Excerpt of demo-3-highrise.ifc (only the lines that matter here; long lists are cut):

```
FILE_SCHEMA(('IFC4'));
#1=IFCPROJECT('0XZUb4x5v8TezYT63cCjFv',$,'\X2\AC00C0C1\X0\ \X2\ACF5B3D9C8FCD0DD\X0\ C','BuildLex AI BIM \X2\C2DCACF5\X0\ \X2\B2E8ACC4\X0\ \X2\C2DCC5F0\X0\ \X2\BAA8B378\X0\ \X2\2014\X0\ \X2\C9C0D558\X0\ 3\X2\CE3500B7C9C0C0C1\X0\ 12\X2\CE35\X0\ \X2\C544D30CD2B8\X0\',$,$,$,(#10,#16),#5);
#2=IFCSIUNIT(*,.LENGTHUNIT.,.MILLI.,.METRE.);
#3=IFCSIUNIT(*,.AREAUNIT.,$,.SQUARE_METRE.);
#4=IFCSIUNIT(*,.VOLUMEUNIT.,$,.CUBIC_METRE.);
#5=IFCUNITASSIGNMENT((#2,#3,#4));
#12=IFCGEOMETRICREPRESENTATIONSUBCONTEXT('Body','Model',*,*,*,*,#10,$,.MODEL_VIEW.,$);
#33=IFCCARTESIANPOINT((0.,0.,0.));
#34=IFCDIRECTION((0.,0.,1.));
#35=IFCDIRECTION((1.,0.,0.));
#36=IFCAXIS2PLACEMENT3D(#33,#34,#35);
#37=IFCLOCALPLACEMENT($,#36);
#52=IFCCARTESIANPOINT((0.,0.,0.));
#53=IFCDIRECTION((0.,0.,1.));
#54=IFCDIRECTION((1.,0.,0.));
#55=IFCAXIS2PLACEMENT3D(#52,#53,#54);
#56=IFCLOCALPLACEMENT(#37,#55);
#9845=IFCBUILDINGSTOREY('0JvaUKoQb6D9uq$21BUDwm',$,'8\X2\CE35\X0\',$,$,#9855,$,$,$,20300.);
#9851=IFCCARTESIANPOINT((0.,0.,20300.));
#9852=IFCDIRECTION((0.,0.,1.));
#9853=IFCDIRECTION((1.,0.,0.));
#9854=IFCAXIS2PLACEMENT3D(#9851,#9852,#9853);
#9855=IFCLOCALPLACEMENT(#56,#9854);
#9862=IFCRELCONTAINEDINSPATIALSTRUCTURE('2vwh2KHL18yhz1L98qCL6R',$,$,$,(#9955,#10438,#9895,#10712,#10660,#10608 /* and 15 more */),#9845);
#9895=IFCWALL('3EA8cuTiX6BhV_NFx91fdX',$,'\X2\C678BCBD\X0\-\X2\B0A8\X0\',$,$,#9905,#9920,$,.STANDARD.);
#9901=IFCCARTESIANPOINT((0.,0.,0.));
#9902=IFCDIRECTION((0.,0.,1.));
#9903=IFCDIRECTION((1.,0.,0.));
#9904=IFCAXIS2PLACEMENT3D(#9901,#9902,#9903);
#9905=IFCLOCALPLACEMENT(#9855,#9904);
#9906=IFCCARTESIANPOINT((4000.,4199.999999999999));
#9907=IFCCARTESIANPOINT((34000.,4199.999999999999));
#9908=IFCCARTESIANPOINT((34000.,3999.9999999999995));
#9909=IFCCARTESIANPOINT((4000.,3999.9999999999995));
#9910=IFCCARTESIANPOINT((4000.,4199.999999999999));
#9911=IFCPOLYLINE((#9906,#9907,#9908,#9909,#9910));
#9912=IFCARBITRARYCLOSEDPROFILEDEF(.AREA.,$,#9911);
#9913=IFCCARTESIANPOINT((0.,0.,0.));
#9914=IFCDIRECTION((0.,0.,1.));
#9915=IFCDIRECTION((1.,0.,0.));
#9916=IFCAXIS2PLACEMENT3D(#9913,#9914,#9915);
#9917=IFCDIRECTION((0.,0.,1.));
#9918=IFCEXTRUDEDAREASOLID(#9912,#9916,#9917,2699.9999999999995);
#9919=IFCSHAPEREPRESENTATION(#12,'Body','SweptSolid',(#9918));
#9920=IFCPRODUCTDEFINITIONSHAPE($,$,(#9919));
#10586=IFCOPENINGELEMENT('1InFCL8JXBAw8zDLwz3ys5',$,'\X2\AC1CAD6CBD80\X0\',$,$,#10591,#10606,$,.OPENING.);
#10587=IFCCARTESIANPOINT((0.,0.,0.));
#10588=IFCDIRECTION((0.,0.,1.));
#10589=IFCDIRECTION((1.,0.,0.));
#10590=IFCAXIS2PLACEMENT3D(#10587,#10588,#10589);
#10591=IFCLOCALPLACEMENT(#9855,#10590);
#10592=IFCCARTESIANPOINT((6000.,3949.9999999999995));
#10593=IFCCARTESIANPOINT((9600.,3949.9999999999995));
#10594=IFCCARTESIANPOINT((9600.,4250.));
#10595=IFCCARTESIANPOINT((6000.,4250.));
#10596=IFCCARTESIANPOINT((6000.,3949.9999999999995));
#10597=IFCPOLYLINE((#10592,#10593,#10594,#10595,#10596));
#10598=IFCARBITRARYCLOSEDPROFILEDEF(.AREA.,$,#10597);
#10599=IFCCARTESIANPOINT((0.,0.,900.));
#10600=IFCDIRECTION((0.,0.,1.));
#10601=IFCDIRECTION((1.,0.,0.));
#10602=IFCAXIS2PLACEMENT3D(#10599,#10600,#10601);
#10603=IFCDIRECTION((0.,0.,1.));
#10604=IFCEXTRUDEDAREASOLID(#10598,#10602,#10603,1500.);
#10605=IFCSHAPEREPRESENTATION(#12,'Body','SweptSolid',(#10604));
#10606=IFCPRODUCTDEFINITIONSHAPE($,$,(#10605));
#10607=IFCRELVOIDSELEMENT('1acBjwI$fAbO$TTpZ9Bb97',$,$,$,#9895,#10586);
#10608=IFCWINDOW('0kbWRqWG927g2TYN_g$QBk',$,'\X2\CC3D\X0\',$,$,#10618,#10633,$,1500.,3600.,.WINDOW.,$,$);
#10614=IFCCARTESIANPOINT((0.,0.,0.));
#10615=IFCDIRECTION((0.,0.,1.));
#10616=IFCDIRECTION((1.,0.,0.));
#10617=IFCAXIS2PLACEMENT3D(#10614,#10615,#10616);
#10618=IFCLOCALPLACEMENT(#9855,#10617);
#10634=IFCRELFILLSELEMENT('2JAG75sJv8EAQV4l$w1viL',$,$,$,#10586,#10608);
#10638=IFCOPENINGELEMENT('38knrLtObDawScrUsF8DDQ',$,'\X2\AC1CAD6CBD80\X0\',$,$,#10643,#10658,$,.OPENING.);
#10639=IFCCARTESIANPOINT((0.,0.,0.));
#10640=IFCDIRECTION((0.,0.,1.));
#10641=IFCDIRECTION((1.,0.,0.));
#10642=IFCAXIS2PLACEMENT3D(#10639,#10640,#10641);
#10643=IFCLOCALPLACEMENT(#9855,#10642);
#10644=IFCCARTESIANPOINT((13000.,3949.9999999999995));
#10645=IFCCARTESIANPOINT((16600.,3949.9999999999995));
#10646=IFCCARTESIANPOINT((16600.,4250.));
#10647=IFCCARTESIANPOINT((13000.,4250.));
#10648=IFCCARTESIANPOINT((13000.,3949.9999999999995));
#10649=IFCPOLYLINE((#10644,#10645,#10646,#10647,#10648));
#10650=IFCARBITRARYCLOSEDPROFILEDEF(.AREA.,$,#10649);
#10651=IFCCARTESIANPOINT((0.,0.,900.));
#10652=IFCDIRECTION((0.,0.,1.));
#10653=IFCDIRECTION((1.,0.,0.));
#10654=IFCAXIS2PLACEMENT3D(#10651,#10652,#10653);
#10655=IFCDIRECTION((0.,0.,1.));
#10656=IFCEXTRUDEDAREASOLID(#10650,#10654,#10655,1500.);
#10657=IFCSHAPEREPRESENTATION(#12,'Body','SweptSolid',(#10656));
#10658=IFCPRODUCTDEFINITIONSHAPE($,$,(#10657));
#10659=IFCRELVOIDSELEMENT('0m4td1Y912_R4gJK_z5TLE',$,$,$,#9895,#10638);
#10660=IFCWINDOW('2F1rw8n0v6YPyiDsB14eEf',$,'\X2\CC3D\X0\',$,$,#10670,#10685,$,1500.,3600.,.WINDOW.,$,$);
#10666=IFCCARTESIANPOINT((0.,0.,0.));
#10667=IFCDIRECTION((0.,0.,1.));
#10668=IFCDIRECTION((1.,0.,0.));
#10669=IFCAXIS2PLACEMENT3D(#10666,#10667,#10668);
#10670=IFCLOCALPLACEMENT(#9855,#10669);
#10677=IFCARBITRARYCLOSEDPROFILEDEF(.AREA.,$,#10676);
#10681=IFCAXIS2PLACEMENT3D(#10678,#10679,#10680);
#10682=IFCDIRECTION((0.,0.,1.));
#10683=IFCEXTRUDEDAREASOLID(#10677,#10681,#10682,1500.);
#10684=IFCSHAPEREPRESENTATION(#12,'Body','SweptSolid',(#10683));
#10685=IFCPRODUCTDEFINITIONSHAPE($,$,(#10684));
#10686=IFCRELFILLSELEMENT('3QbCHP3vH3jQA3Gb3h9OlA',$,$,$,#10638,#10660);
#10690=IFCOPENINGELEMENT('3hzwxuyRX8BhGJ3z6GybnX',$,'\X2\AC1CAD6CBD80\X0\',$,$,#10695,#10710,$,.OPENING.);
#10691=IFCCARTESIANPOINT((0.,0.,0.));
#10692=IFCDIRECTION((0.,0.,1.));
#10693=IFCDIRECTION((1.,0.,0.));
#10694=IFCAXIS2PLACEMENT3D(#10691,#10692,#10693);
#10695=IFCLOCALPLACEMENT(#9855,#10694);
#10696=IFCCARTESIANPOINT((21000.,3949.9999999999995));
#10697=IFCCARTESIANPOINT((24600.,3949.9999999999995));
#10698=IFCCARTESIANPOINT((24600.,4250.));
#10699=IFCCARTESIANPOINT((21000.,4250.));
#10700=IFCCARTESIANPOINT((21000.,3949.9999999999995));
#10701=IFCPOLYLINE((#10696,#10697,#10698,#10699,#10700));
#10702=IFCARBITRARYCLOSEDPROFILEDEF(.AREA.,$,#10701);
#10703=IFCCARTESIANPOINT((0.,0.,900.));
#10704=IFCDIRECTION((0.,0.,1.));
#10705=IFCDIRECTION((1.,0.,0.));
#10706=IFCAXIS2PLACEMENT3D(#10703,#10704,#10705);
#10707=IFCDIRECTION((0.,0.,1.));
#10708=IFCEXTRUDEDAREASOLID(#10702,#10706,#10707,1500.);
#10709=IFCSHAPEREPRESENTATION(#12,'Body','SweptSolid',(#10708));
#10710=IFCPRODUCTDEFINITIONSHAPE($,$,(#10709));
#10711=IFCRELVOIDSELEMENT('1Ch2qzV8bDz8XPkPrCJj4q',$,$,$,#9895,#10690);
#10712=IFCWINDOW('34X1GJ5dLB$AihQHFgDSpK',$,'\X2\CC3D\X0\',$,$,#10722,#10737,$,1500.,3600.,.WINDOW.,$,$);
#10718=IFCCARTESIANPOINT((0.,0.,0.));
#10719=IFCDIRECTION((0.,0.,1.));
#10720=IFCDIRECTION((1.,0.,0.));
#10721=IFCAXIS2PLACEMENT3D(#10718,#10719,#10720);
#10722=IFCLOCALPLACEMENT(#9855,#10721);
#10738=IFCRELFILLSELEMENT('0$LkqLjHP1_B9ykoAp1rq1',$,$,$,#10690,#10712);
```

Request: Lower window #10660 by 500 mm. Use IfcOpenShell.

```python
import numpy as np
import ifcopenshell
import ifcopenshell.api.geometry
import ifcopenshell.util.placement
import ifcopenshell.util.unit

model = ifcopenshell.open("demo-3-highrise.ifc")
unit_scale = ifcopenshell.util.unit.calculate_unit_scale(model)

window = model.by_guid("2F1rw8n0v6YPyiDsB14eEf")
opening = window.FillsVoids[0].RelatingOpeningElement
dz = -500.0

shift = np.array([0.0, 0.0, dz])
# The window is not placed relative to its opening, so move both.
for product in (opening, window):
    matrix = ifcopenshell.util.placement.get_local_placement(product.ObjectPlacement)
    matrix[:3, 3] += shift
    ifcopenshell.api.geometry.edit_object_placement(model, product=product, matrix=matrix, is_si=False)

print(f"moved by {dz * unit_scale:+.3f} m")

model.write("demo-3-highrise_edited.ifc")
```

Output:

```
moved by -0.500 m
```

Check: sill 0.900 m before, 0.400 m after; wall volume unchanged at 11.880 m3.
